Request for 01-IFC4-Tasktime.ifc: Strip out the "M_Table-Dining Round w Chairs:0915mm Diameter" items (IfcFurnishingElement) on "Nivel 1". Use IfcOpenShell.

First a look at what the model holds.

```python
import ifcopenshell
import ifcopenshell.util.element

model = ifcopenshell.open("01-IFC4-Tasktime.ifc")
print(model.schema)
storey = next(s for s in model.by_type("IfcBuildingStorey") if s.Name == "Nivel 1")
furniture = [e for e in ifcopenshell.util.element.get_decomposition(storey) if e.is_a("IfcFurnishingElement")]
seen = {}
for e in furniture:
    element_type = ifcopenshell.util.element.get_type(e)
    name = element_type.Name if element_type not in (None, e) else None
    seen[name] = seen.get(name, 0) + 1
for name, count in sorted(seen.items(), key=str):
    print(count, "x", name)
```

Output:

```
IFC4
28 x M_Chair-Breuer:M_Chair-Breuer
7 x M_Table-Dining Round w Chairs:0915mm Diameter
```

```python
import ifcopenshell
import ifcopenshell.api.root
import ifcopenshell.util.element

model = ifcopenshell.open("01-IFC4-Tasktime.ifc")

storey = next(s for s in model.by_type("IfcBuildingStorey") if s.Name == "Nivel 1")
furniture = [e for e in ifcopenshell.util.element.get_decomposition(storey) if e.is_a("IfcFurnishingElement")]
targets = [e for e in furniture if (t := ifcopenshell.util.element.get_type(e)) not in (None, e) and t.Name == "M_Table-Dining Round w Chairs:0915mm Diameter"]

for e in targets:
    ifcopenshell.api.root.remove_product(model, product=e)
print(len(targets), "removed")

model.write("01-IFC4-Tasktime_edited.ifc")
```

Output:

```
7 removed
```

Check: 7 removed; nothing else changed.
